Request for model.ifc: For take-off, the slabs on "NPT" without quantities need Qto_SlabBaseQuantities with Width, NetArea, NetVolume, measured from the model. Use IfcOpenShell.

First a look at what the model holds.

```python
import ifcopenshell
import ifcopenshell.util.element
import ifcopenshell.util.unit

model = ifcopenshell.open("model.ifc")
print(model.schema)
for unit_type in ("LENGTHUNIT", "AREAUNIT", "VOLUMEUNIT"):
    print(unit_type, ifcopenshell.util.unit.calculate_unit_scale(model, unit_type))
storey = next(s for s in model.by_type("IfcBuildingStorey") if s.Name == "NPT")
slabs = [e for e in ifcopenshell.util.element.get_decomposition(storey) if e.is_a("IfcSlab")]
for e in sorted(slabs, key=lambda e: e.id()):
    print(e.id(), e.is_a(), e.Name, list(ifcopenshell.util.element.get_psets(e, qtos_only=True)), sep=" | ")
```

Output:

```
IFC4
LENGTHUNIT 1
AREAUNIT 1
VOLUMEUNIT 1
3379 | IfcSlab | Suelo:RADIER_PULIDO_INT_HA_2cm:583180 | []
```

```python
import ifcopenshell
import ifcopenshell.api.pset
import ifcopenshell.geom
import ifcopenshell.util.element
import ifcopenshell.util.shape
import ifcopenshell.util.unit

model = ifcopenshell.open("model.ifc")
unit_scale = ifcopenshell.util.unit.calculate_unit_scale(model)
area_scale = ifcopenshell.util.unit.calculate_unit_scale(model, "AREAUNIT")
volume_scale = ifcopenshell.util.unit.calculate_unit_scale(model, "VOLUMEUNIT")
settings = ifcopenshell.geom.settings()

storey = next(s for s in model.by_type("IfcBuildingStorey") if s.Name == "NPT")
slabs = [e for e in ifcopenshell.util.element.get_decomposition(storey) if e.is_a("IfcSlab")]

for e in sorted(slabs, key=lambda e: e.id()):
    if ifcopenshell.util.element.get_psets(e, qtos_only=True, should_inherit=False):
        continue
    # Geometry comes back in metres, in the element's own axes.
    shape = ifcopenshell.geom.create_shape(settings, e)
    values = {
        "Width": ifcopenshell.util.shape.get_z(shape.geometry) / unit_scale,
        "NetArea": ifcopenshell.util.shape.get_footprint_area(shape.geometry) / area_scale,
        "NetVolume": ifcopenshell.util.shape.get_volume(shape.geometry) / volume_scale,
    }
    qto = ifcopenshell.api.pset.add_qto(model, product=e, name="Qto_SlabBaseQuantities")
    ifcopenshell.api.pset.edit_qto(model, qto=qto, properties=values)
    print(e.id(), {k: round(v, 3) for k, v in values.items()})

model.write("model_v2.ifc")
```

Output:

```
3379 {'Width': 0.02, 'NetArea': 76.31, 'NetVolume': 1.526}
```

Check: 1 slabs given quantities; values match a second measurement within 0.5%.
